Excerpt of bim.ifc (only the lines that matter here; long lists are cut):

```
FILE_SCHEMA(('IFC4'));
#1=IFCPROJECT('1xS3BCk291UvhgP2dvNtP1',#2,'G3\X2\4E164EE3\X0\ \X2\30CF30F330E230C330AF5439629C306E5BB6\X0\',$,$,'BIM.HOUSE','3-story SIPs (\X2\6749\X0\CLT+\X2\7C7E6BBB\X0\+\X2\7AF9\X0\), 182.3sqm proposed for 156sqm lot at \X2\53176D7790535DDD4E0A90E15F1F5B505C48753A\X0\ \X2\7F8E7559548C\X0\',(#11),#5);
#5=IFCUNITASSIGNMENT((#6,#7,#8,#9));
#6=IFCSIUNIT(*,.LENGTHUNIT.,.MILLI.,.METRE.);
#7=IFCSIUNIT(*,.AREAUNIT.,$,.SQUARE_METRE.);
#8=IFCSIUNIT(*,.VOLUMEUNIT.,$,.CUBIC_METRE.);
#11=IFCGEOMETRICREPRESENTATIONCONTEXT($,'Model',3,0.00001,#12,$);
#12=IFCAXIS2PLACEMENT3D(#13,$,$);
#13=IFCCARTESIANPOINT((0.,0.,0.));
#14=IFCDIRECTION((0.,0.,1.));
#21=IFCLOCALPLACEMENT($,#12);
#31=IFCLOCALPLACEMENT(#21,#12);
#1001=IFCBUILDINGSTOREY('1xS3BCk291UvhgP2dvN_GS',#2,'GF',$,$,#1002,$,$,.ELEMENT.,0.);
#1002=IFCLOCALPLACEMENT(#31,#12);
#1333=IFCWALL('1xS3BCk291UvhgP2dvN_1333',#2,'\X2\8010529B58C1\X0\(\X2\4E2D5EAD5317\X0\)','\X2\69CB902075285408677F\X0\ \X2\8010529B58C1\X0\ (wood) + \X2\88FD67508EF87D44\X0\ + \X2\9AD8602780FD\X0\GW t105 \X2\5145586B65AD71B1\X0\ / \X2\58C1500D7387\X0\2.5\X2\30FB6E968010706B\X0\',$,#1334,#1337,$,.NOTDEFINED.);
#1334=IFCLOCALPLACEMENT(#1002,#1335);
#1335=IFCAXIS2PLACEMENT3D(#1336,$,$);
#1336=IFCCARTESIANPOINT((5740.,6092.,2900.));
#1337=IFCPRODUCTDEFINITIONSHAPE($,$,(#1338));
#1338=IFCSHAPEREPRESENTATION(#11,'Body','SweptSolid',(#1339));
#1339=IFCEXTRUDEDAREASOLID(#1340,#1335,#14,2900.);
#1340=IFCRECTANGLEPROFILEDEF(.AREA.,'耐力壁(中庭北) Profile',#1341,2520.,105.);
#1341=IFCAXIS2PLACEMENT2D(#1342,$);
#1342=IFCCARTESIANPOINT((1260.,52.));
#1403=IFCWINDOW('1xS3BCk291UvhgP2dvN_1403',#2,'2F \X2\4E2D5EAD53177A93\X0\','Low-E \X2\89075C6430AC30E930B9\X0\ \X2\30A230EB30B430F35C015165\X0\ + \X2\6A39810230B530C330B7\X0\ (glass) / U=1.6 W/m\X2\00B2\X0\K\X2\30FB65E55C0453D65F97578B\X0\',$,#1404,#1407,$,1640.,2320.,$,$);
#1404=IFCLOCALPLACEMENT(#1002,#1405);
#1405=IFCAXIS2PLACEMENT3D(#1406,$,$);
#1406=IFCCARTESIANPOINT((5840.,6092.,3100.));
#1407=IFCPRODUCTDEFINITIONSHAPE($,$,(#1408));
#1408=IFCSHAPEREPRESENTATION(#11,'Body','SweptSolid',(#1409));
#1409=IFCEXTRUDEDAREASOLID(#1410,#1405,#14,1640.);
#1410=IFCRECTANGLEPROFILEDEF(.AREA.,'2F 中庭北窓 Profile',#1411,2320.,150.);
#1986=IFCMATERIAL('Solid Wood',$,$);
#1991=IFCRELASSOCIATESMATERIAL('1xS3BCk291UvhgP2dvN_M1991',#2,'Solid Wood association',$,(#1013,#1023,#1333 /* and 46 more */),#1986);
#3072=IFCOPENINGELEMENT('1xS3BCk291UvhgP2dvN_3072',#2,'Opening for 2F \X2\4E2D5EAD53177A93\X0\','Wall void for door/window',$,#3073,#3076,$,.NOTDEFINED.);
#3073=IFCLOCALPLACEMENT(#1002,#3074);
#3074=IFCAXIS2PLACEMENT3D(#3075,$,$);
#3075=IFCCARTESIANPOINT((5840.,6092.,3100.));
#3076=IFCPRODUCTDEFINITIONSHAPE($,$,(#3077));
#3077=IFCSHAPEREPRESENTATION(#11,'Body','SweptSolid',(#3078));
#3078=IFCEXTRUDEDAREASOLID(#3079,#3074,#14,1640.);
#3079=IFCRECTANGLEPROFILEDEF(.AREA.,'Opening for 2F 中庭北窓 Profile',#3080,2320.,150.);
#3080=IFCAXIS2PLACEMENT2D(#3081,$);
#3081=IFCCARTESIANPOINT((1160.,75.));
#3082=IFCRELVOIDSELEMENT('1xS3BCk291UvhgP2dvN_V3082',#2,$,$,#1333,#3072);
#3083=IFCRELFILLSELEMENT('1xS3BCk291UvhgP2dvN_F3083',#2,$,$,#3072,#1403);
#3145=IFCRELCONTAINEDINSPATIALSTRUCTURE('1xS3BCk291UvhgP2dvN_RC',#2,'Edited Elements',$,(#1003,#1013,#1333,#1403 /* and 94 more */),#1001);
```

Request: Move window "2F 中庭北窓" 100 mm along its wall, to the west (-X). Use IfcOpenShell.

```python
import ifcopenshell
import ifcopenshell.api.geometry
import ifcopenshell.util.placement
import ifcopenshell.util.unit

model = ifcopenshell.open("bim.ifc")
unit_scale = ifcopenshell.util.unit.calculate_unit_scale(model)

window = model.by_guid("1xS3BCk291UvhgP2dvN_1403")
opening = window.FillsVoids[0].RelatingOpeningElement
wall = opening.VoidsElements[0].RelatingBuildingElement

wall_matrix = ifcopenshell.util.placement.get_local_placement(wall.ObjectPlacement)
shift = wall_matrix[:3, 0] * -0.1 / unit_scale
before = ifcopenshell.util.placement.get_local_placement(window.ObjectPlacement)[:3, 3].copy()

# The window is not placed relative to its opening, so move both.
for product in (opening, window):
    matrix = ifcopenshell.util.placement.get_local_placement(product.ObjectPlacement)
    matrix[:3, 3] += shift
    ifcopenshell.api.geometry.edit_object_placement(model, product=product, matrix=matrix, is_si=False)

after = ifcopenshell.util.placement.get_local_placement(window.ObjectPlacement)[:3, 3]
print("window moved by", (after - before).round(3) + 0.0)

model.write("bim_edited.ifc")
```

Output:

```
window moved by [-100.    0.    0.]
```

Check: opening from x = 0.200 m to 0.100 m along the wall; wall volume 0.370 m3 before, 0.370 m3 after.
